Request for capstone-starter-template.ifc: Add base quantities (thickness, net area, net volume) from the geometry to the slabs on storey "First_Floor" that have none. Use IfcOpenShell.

First a look at what the model holds.

```python
import ifcopenshell
import ifcopenshell.util.element
import ifcopenshell.util.unit

model = ifcopenshell.open("capstone-starter-template.ifc")
print(model.schema)
for unit_type in ("LENGTHUNIT", "AREAUNIT", "VOLUMEUNIT"):
    print(unit_type, ifcopenshell.util.unit.calculate_unit_scale(model, unit_type))
storey = next(s for s in model.by_type("IfcBuildingStorey") if s.Name == "First_Floor")
slabs = [e for e in ifcopenshell.util.element.get_decomposition(storey) if e.is_a("IfcSlab")]
for e in sorted(slabs, key=lambda e: e.id()):
    print(e.id(), e.is_a(), e.Name, list(ifcopenshell.util.element.get_psets(e, qtos_only=True)), sep=" | ")
```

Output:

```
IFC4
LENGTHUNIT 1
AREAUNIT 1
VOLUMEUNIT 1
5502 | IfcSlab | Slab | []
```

```python
import ifcopenshell
import ifcopenshell.api.pset
import ifcopenshell.geom
import ifcopenshell.util.element
import ifcopenshell.util.shape
import ifcopenshell.util.unit

model = ifcopenshell.open("capstone-starter-template.ifc")
unit_scale = ifcopenshell.util.unit.calculate_unit_scale(model)
area_scale = ifcopenshell.util.unit.calculate_unit_scale(model, "AREAUNIT")
volume_scale = ifcopenshell.util.unit.calculate_unit_scale(model, "VOLUMEUNIT")
settings = ifcopenshell.geom.settings()

storey = next(s for s in model.by_type("IfcBuildingStorey") if s.Name == "First_Floor")
slabs = [e for e in ifcopenshell.util.element.get_decomposition(storey) if e.is_a("IfcSlab")]

for e in sorted(slabs, key=lambda e: e.id()):
    if ifcopenshell.util.element.get_psets(e, qtos_only=True, should_inherit=False):
        continue
    # Geometry comes back in metres, in the element's own axes.
    shape = ifcopenshell.geom.create_shape(settings, e)
    values = {
        "Width": ifcopenshell.util.shape.get_z(shape.geometry) / unit_scale,
        "NetArea": ifcopenshell.util.shape.get_footprint_area(shape.geometry) / area_scale,
        "NetVolume": ifcopenshell.util.shape.get_volume(shape.geometry) / volume_scale,
    }
    qto = ifcopenshell.api.pset.add_qto(model, product=e, name="Qto_SlabBaseQuantities")
    ifcopenshell.api.pset.edit_qto(model, qto=qto, properties=values)
    print(e.id(), {k: round(v, 3) for k, v in values.items()})

model.write("capstone-starter-template_v2.ifc")
```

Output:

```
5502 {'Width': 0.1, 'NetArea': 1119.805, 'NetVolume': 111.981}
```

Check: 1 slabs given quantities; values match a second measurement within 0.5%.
